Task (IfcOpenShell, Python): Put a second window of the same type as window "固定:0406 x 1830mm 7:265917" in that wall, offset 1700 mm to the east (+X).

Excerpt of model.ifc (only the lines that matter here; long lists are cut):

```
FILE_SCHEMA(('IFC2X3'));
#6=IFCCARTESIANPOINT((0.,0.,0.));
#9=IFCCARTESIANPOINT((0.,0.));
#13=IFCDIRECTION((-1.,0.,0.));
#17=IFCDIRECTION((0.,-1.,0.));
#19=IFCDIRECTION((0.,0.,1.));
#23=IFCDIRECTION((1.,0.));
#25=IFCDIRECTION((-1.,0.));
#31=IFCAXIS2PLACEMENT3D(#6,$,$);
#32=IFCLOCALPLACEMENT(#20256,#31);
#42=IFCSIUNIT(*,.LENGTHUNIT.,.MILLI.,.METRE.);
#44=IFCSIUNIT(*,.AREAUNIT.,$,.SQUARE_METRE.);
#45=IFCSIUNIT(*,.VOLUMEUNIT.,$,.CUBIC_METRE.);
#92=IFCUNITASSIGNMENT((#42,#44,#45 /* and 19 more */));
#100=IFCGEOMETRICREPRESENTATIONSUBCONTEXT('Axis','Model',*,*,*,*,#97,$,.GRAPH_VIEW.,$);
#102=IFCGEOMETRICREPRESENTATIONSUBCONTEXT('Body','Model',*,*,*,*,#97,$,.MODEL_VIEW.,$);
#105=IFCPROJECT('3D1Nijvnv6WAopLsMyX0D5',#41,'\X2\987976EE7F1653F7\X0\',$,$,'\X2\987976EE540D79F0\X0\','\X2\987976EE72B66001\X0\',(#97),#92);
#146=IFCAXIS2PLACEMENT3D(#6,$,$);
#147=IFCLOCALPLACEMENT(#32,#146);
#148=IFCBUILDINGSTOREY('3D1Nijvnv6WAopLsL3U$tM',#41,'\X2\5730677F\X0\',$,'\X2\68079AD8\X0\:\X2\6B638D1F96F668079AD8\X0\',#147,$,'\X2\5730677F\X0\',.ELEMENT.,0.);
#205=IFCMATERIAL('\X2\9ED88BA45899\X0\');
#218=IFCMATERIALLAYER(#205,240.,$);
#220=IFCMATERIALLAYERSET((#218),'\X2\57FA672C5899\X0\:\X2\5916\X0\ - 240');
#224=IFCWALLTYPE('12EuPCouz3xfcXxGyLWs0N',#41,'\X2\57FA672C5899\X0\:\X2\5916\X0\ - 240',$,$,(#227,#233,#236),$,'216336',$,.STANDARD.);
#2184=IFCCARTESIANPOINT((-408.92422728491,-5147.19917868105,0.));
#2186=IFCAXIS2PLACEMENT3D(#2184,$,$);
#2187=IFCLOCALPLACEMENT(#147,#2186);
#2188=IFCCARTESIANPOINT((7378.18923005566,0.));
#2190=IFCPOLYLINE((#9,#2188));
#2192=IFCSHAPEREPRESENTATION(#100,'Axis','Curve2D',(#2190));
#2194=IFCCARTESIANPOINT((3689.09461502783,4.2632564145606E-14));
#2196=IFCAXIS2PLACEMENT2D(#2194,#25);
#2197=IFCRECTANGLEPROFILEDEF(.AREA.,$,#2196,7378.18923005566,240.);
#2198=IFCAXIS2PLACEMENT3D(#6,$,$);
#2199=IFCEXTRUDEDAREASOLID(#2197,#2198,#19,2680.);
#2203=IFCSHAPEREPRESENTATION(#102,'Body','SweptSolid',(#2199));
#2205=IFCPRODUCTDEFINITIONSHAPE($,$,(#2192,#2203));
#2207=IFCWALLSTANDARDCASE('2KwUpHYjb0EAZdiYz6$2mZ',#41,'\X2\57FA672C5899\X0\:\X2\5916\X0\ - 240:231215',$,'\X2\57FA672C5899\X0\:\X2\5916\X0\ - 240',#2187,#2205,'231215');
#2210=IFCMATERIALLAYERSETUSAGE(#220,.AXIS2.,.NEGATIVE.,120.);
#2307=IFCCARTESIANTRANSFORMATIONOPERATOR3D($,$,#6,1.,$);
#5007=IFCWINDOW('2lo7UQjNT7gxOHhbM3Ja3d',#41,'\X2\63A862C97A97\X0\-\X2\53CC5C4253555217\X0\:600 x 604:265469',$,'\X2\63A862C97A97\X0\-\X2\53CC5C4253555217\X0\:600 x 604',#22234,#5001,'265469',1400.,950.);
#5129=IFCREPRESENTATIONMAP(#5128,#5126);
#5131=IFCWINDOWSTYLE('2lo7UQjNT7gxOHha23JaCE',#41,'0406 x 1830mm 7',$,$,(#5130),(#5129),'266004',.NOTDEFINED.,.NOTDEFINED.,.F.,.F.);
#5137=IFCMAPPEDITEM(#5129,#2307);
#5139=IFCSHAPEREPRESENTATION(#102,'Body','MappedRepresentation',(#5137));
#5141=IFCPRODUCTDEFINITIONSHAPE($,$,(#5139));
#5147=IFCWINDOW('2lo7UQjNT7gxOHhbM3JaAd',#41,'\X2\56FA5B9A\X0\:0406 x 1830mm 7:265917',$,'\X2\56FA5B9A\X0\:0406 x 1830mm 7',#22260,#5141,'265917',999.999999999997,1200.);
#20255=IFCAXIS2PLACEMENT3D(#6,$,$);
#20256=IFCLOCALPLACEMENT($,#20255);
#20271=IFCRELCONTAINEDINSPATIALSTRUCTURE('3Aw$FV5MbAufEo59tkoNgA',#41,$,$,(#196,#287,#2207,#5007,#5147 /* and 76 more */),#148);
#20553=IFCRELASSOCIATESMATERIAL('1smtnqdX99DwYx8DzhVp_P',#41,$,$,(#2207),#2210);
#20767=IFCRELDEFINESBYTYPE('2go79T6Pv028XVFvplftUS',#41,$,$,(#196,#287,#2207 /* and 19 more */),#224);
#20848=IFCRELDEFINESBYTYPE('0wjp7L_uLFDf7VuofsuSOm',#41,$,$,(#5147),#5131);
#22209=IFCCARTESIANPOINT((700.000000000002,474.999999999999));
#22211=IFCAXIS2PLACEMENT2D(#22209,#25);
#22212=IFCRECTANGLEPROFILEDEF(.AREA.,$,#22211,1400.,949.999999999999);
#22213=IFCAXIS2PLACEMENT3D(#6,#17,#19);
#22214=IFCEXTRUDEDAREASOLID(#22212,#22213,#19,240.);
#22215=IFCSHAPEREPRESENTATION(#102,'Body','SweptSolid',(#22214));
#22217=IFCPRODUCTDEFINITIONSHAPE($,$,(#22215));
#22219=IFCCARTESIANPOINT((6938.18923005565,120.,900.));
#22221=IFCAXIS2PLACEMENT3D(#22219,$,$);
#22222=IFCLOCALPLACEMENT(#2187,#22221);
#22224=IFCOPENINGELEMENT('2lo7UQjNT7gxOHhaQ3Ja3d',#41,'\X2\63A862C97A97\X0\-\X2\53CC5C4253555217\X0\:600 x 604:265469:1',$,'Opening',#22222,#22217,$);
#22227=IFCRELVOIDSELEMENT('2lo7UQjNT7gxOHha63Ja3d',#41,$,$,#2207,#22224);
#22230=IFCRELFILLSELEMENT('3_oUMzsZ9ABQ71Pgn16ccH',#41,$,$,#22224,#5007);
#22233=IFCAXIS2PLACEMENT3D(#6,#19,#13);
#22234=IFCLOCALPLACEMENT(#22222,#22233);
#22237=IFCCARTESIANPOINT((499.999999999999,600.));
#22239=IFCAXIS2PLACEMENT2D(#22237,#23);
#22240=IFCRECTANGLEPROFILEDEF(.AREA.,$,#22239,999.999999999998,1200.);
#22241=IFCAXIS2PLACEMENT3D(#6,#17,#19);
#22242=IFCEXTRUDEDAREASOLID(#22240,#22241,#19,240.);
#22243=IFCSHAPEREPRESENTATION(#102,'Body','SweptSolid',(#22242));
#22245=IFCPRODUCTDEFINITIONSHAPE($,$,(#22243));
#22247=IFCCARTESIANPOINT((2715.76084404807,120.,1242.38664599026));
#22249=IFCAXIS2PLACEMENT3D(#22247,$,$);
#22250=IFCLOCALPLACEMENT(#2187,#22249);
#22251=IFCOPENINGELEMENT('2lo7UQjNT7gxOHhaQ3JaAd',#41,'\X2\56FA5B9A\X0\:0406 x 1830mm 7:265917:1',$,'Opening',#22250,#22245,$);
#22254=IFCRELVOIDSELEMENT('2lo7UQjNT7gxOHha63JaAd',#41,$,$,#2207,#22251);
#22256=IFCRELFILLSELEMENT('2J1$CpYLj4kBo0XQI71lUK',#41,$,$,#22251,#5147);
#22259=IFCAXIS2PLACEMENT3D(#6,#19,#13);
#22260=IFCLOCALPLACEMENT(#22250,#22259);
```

```python
import ifcopenshell
import ifcopenshell.api.feature
import ifcopenshell.api.geometry
import ifcopenshell.api.root
import ifcopenshell.geom
import ifcopenshell.util.element
import ifcopenshell.util.placement
import ifcopenshell.util.shape
import ifcopenshell.util.unit

model = ifcopenshell.open("model.ifc")
unit_scale = ifcopenshell.util.unit.calculate_unit_scale(model)
settings = ifcopenshell.geom.settings()


def volume(element):
    """Net volume in cubic metres, openings subtracted."""
    shape = ifcopenshell.geom.create_shape(settings, element)
    return ifcopenshell.util.shape.get_volume(shape.geometry)


def reuse_history(source, copy):
    """copy_class also copies each property set's owner history, people and application; keep the originals."""
    for rel in copy.IsDefinedBy:
        if rel.is_a("IfcRelDefinesByProperties") and (history := rel.RelatingPropertyDefinition.OwnerHistory):
            rel.RelatingPropertyDefinition.OwnerHistory = source.OwnerHistory
            ifcopenshell.util.element.remove_deep2(model, history)


window = model.by_guid("2lo7UQjNT7gxOHhbM3JaAd")
opening = window.FillsVoids[0].RelatingOpeningElement
wall = opening.VoidsElements[0].RelatingBuildingElement
before = volume(wall)
shift = ifcopenshell.util.placement.get_local_placement(wall.ObjectPlacement)[:3, 0] * 1.7 / unit_scale

# copy_class copies the void relationship, type, container and properties, but no geometry.
new_opening = ifcopenshell.api.root.copy_class(model, product=opening)
new_opening.Representation = ifcopenshell.util.element.copy_deep(
    model, opening.Representation, exclude=["IfcGeometricRepresentationContext", "IfcRepresentationMap"]
)
new_opening.Name = "固定:0406 x 1830mm 7"
new_window = ifcopenshell.api.root.copy_class(model, product=window)
new_window.Representation = ifcopenshell.util.element.copy_deep(
    model, window.Representation, exclude=["IfcGeometricRepresentationContext", "IfcRepresentationMap"]
)
new_window.Name = "固定:0406 x 1830mm 7"
new_window.Tag = None
reuse_history(window, new_window)
fills = ifcopenshell.api.feature.add_filling(model, opening=new_opening, element=new_window)
fills.OwnerHistory = new_window.OwnerHistory  # required in IFC2X3

for old, new in ((opening, new_opening), (window, new_window)):
    matrix = ifcopenshell.util.placement.get_local_placement(old.ObjectPlacement)
    matrix[:3, 3] += shift
    ifcopenshell.api.geometry.edit_object_placement(model, product=new, matrix=matrix, is_si=False)

after = volume(wall)

print(f"wall volume {before:.3f} -> {after:.3f} m3")

model.write("model_edited.ifc")
```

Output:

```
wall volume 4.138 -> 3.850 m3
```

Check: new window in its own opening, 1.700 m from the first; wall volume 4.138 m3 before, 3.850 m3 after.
